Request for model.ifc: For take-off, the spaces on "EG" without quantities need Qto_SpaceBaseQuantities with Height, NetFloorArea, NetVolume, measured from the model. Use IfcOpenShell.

First a look at what the model holds.

```python
import ifcopenshell
import ifcopenshell.util.element
import ifcopenshell.util.unit

model = ifcopenshell.open("model.ifc")
print(model.schema)
for unit_type in ("LENGTHUNIT", "AREAUNIT", "VOLUMEUNIT"):
    print(unit_type, ifcopenshell.util.unit.calculate_unit_scale(model, unit_type))
storey = next(s for s in model.by_type("IfcBuildingStorey") if s.Name == "EG")
spaces = [e for e in ifcopenshell.util.element.get_decomposition(storey) if e.is_a("IfcSpace")]
for e in sorted(spaces, key=lambda e: e.id()):
    print(e.id(), e.is_a(), e.Name, list(ifcopenshell.util.element.get_psets(e, qtos_only=True)), sep=" | ")
```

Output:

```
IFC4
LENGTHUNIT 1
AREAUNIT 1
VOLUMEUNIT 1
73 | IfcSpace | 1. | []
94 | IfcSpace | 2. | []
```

```python
import ifcopenshell
import ifcopenshell.api.pset
import ifcopenshell.geom
import ifcopenshell.util.element
import ifcopenshell.util.shape
import ifcopenshell.util.unit

model = ifcopenshell.open("model.ifc")
unit_scale = ifcopenshell.util.unit.calculate_unit_scale(model)
area_scale = ifcopenshell.util.unit.calculate_unit_scale(model, "AREAUNIT")
volume_scale = ifcopenshell.util.unit.calculate_unit_scale(model, "VOLUMEUNIT")
settings = ifcopenshell.geom.settings()

storey = next(s for s in model.by_type("IfcBuildingStorey") if s.Name == "EG")
spaces = [e for e in ifcopenshell.util.element.get_decomposition(storey) if e.is_a("IfcSpace")]

for e in sorted(spaces, key=lambda e: e.id()):
    if ifcopenshell.util.element.get_psets(e, qtos_only=True, should_inherit=False):
        continue
    # Geometry comes back in metres, in the element's own axes.
    shape = ifcopenshell.geom.create_shape(settings, e)
    values = {
        "Height": ifcopenshell.util.shape.get_z(shape.geometry) / unit_scale,
        "NetFloorArea": ifcopenshell.util.shape.get_footprint_area(shape.geometry) / area_scale,
        "NetVolume": ifcopenshell.util.shape.get_volume(shape.geometry) / volume_scale,
    }
    qto = ifcopenshell.api.pset.add_qto(model, product=e, name="Qto_SpaceBaseQuantities")
    ifcopenshell.api.pset.edit_qto(model, qto=qto, properties=values)
    print(e.id(), {k: round(v, 3) for k, v in values.items()})

model.write("model-out.ifc")
```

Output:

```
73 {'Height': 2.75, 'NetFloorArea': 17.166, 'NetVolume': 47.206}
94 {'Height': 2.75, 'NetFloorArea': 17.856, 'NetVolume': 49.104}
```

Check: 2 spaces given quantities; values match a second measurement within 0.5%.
